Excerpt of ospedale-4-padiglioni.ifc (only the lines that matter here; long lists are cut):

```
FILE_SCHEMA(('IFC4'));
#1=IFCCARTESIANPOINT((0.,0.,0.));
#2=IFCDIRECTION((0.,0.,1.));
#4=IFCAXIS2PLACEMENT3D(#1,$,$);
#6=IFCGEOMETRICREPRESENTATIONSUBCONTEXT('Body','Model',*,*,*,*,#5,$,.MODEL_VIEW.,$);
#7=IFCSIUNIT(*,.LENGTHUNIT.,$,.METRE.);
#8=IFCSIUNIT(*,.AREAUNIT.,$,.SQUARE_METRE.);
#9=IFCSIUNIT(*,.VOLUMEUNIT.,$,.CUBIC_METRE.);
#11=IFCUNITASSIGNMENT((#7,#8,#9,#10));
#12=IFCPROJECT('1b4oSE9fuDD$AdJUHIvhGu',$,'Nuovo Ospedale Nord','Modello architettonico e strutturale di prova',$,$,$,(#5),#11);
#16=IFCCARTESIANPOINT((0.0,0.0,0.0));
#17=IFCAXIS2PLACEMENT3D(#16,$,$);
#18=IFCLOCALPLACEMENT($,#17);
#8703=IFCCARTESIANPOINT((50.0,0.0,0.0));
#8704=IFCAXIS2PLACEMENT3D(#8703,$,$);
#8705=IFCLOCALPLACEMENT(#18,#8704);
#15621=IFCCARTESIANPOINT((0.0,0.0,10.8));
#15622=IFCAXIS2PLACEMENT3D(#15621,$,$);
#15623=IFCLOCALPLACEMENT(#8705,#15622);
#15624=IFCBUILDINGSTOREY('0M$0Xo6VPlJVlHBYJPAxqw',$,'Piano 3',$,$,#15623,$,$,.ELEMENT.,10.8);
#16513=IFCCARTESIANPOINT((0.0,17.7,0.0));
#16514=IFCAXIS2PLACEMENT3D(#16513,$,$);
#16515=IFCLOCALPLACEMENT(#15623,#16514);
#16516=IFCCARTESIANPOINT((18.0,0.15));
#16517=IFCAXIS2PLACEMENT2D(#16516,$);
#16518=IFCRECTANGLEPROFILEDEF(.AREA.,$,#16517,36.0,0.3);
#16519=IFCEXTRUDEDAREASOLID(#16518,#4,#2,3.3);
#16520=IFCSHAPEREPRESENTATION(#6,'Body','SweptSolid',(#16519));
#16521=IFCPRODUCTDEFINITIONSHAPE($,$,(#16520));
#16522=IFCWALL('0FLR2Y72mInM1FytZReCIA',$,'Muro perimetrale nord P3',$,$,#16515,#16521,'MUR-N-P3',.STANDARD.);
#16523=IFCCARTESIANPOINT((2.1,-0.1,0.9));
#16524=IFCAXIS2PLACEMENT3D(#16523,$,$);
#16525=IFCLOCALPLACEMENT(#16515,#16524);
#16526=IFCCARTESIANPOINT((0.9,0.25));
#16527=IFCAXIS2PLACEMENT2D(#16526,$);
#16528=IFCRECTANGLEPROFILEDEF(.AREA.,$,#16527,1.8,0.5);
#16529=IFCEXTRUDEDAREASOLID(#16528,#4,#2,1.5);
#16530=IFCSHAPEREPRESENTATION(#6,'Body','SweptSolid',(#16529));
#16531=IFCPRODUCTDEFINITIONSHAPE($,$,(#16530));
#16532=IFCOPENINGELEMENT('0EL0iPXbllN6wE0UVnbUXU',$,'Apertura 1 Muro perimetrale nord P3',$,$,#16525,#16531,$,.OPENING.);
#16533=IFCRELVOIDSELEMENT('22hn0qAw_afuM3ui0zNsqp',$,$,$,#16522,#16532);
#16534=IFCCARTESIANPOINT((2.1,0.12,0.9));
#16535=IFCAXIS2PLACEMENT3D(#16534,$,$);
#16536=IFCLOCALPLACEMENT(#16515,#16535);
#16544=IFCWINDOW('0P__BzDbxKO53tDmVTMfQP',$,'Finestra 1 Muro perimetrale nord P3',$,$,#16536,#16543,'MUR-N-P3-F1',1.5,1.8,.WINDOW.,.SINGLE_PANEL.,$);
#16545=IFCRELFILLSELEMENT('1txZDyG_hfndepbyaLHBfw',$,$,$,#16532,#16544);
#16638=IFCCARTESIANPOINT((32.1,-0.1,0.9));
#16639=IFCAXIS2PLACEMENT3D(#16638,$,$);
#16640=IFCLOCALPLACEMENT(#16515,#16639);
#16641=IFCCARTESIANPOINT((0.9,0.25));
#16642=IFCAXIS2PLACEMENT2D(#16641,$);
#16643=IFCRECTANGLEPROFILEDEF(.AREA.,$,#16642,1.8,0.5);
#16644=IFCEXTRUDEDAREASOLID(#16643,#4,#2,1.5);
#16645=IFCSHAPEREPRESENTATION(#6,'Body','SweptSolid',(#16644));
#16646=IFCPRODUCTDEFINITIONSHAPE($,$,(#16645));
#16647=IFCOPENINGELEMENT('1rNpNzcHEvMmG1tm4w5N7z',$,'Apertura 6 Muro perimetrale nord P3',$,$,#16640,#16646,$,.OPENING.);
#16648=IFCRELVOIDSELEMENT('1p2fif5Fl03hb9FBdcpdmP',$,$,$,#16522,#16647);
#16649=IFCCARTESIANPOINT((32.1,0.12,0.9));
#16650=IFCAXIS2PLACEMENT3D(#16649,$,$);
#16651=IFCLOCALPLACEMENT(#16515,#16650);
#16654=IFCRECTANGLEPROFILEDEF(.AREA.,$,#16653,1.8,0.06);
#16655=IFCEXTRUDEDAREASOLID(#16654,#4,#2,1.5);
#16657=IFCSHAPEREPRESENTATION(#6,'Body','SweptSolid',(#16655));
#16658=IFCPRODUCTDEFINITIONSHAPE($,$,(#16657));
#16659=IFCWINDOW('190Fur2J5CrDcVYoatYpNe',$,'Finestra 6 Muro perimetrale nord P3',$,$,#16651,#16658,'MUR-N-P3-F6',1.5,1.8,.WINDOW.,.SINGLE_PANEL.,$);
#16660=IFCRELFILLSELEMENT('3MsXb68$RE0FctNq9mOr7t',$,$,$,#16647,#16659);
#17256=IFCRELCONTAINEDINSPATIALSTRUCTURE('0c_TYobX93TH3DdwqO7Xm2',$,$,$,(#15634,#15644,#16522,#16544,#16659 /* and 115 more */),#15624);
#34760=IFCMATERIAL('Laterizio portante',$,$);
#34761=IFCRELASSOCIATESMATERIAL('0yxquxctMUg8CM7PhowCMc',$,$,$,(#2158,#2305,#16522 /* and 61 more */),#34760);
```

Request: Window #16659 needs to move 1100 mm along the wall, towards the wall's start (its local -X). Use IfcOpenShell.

```python
import ifcopenshell
import ifcopenshell.api.geometry
import ifcopenshell.util.placement

model = ifcopenshell.open("ospedale-4-padiglioni.ifc")

window = model.by_guid("190Fur2J5CrDcVYoatYpNe")
opening = window.FillsVoids[0].RelatingOpeningElement
wall = opening.VoidsElements[0].RelatingBuildingElement

wall_matrix = ifcopenshell.util.placement.get_local_placement(wall.ObjectPlacement)
shift = wall_matrix[:3, 0] * -1.1
before = ifcopenshell.util.placement.get_local_placement(window.ObjectPlacement)[:3, 3].copy()

# The window is not placed relative to its opening, so move both.
for product in (opening, window):
    matrix = ifcopenshell.util.placement.get_local_placement(product.ObjectPlacement)
    matrix[:3, 3] += shift
    ifcopenshell.api.geometry.edit_object_placement(model, product=product, matrix=matrix, is_si=False)

after = ifcopenshell.util.placement.get_local_placement(window.ObjectPlacement)[:3, 3]
print("window moved by", (after - before).round(3) + 0.0)

model.write("ospedale-4-padiglioni_v2.ifc")
```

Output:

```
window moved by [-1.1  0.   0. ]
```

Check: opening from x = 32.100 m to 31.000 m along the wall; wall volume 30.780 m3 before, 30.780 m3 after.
